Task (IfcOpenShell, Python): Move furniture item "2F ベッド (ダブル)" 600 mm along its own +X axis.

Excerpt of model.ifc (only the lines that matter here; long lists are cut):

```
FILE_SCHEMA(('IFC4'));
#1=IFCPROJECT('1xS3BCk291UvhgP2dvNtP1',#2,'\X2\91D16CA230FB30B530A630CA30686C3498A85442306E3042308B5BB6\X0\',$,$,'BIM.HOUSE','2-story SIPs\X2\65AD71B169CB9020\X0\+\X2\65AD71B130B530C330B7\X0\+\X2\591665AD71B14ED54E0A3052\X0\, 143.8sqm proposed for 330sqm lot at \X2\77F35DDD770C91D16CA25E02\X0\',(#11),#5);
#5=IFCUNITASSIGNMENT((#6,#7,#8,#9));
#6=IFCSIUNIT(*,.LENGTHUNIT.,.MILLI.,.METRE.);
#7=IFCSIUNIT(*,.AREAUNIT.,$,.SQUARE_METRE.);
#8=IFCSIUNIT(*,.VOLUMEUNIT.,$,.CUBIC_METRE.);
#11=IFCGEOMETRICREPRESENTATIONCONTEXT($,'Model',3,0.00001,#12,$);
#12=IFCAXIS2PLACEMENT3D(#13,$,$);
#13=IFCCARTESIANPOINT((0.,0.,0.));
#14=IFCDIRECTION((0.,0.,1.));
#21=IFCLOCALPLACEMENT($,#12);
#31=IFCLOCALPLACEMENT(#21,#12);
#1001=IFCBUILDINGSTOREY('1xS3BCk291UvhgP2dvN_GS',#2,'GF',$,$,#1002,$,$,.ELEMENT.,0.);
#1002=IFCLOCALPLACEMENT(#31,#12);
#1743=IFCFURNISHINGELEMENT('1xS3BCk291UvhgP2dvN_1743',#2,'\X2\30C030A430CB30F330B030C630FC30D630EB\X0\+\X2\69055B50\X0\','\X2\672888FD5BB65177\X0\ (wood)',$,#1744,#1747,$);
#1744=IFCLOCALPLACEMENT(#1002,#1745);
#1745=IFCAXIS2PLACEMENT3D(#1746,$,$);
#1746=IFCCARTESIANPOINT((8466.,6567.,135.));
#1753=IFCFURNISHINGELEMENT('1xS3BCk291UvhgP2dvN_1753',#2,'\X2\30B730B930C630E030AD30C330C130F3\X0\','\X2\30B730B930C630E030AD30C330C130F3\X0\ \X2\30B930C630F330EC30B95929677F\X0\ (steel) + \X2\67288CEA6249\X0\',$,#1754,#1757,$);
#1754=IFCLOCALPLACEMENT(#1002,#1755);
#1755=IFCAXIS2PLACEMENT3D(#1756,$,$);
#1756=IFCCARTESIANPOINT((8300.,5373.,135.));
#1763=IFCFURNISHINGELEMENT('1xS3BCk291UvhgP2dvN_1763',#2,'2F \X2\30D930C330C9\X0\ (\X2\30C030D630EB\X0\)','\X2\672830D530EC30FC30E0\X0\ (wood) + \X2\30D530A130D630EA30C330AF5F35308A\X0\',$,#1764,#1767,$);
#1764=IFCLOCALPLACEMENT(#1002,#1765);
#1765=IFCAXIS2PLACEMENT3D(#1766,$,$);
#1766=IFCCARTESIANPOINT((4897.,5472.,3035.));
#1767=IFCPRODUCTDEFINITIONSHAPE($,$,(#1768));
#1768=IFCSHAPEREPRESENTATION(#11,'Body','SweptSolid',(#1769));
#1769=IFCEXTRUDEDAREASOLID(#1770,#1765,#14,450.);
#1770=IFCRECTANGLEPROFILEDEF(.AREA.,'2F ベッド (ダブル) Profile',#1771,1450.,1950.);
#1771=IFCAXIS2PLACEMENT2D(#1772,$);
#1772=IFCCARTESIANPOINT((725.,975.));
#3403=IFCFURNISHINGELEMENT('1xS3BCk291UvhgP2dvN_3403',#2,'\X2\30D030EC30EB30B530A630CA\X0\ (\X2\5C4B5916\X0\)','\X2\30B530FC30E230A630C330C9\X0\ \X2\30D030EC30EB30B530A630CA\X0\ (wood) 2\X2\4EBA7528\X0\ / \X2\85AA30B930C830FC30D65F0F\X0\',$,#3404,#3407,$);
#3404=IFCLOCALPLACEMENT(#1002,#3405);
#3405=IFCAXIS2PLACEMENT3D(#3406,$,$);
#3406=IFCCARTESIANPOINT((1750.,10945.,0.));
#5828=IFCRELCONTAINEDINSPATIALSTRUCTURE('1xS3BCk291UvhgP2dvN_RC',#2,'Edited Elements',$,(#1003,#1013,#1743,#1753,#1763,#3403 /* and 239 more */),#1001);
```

```python
import ifcopenshell
import ifcopenshell.api.geometry
import ifcopenshell.util.placement
import ifcopenshell.util.unit

model = ifcopenshell.open("model.ifc")
unit_scale = ifcopenshell.util.unit.calculate_unit_scale(model)

item = model.by_guid("1xS3BCk291UvhgP2dvN_1763")
matrix = ifcopenshell.util.placement.get_local_placement(item.ObjectPlacement)
matrix[:3, 3] += matrix[:3, 0] * 0.6 / unit_scale
ifcopenshell.api.geometry.edit_object_placement(model, product=item, matrix=matrix, is_si=False)

print(ifcopenshell.util.placement.get_local_placement(item.ObjectPlacement).round(3) + 0.0)

model.write("model_edited.ifc")
```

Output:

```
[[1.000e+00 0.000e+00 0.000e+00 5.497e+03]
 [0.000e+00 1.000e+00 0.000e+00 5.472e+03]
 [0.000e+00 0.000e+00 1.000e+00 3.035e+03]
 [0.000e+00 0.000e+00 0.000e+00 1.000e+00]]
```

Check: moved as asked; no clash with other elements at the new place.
